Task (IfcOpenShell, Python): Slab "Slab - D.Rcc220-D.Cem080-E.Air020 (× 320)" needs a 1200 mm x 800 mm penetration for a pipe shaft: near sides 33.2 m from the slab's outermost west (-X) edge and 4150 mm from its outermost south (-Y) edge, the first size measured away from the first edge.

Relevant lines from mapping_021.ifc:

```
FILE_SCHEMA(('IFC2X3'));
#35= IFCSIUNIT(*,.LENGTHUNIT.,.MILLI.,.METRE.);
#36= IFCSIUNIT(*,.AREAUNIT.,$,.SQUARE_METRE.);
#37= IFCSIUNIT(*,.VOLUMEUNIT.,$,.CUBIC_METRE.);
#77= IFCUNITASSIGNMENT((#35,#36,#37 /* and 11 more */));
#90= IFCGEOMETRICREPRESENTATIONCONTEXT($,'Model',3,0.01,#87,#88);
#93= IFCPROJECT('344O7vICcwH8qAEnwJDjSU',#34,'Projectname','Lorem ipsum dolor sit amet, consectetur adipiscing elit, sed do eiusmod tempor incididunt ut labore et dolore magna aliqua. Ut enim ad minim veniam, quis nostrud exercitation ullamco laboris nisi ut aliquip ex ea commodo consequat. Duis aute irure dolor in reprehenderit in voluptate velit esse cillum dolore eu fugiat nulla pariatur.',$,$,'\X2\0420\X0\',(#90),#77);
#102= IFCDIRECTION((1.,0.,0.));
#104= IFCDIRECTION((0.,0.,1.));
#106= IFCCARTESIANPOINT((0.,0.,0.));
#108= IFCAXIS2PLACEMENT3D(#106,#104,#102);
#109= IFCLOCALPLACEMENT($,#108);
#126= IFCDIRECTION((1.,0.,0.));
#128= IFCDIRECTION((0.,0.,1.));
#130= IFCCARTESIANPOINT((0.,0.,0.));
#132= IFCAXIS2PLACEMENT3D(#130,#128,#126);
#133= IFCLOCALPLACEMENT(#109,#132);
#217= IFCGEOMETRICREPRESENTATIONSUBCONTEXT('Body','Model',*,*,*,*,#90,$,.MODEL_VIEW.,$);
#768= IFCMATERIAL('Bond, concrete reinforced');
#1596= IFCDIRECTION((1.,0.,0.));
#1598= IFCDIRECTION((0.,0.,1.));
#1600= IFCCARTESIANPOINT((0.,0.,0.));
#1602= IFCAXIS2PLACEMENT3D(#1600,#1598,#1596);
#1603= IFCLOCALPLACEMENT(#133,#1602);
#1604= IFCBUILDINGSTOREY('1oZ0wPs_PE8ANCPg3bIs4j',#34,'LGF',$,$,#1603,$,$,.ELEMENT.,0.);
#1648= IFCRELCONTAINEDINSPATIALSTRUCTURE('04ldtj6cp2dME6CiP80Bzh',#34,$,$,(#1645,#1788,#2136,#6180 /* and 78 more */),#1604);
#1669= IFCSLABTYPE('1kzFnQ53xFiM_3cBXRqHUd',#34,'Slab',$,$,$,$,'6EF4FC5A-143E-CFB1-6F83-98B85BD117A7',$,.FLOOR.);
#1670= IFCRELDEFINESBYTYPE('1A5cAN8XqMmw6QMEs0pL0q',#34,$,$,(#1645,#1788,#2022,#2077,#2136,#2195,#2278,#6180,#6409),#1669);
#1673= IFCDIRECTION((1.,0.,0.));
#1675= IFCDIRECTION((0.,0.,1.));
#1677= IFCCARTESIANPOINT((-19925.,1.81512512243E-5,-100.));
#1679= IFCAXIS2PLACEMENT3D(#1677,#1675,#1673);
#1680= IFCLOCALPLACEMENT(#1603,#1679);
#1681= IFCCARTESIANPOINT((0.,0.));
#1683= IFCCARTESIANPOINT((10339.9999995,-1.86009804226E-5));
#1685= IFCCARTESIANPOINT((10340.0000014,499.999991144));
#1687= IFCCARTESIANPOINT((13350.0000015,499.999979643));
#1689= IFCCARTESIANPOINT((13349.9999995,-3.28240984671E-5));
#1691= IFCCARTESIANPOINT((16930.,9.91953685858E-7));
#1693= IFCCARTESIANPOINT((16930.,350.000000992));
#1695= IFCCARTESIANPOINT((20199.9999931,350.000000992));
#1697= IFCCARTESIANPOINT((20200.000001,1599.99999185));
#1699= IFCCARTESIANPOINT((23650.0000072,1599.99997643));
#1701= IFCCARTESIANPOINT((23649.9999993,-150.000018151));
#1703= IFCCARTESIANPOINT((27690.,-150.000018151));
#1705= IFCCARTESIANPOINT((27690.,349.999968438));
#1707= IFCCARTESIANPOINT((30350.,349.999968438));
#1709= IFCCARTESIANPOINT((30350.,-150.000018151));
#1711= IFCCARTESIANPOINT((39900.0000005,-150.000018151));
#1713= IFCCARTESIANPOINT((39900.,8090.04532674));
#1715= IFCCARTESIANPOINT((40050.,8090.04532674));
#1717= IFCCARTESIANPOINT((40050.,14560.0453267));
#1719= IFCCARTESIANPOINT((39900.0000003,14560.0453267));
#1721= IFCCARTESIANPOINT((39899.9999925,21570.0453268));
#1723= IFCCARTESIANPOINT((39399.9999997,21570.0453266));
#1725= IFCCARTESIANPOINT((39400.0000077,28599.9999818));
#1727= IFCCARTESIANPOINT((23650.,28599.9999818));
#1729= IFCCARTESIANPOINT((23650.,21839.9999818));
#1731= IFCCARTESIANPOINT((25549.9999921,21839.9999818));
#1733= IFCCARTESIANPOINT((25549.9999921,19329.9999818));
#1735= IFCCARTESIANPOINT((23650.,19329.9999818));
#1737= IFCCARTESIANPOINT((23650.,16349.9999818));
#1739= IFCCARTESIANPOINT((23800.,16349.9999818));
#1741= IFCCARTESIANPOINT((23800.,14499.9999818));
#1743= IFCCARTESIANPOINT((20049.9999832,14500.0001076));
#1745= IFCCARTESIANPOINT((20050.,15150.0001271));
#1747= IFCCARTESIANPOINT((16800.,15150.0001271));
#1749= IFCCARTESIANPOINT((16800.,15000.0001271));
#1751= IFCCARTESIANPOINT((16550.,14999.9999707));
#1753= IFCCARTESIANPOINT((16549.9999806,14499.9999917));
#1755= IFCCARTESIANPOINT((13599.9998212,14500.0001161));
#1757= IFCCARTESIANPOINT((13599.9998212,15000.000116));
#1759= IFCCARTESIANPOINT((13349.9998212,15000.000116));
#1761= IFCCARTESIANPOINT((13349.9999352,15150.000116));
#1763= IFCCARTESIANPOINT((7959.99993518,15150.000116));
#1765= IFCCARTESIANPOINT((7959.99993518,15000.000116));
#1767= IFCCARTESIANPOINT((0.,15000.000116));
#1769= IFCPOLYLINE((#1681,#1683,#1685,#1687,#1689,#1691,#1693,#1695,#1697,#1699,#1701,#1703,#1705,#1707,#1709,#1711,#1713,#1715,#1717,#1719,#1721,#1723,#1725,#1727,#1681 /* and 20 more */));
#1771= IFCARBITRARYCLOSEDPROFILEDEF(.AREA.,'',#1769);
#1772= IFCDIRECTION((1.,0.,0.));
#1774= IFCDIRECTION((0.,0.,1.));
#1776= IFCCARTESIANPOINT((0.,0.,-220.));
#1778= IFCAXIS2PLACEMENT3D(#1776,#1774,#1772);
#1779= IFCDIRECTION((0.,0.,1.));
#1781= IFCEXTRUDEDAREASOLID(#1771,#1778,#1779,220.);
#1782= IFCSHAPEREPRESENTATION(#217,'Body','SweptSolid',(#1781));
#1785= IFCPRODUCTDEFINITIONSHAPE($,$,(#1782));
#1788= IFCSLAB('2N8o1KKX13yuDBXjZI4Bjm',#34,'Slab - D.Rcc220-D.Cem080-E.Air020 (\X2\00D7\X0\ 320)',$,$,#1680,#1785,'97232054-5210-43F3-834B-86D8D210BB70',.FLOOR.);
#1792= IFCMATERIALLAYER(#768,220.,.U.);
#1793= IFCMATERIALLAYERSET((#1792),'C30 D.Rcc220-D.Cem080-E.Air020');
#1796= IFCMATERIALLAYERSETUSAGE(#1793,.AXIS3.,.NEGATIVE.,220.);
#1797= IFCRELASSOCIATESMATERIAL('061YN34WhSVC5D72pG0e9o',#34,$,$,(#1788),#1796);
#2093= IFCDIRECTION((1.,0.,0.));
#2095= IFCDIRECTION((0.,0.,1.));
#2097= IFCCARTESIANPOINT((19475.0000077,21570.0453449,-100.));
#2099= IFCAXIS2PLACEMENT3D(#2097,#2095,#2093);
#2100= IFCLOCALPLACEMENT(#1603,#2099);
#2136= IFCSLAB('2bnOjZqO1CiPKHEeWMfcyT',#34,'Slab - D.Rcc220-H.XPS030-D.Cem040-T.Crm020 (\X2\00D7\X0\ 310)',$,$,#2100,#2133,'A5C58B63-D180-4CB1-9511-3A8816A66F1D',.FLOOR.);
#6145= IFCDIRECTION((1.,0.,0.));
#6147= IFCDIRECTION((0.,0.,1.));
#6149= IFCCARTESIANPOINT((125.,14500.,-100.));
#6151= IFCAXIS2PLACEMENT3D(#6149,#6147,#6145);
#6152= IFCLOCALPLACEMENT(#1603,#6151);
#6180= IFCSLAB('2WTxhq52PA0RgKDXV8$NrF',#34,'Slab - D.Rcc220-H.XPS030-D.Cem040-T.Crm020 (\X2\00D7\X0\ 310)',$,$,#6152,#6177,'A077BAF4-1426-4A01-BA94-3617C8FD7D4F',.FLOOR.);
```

```python
import numpy as np
import ifcopenshell
import ifcopenshell.api.feature
import ifcopenshell.api.geometry
import ifcopenshell.api.root
import ifcopenshell.geom
import ifcopenshell.util.placement
import ifcopenshell.util.representation
import ifcopenshell.util.shape
import ifcopenshell.util.unit

model = ifcopenshell.open("mapping_021.ifc")
unit_scale = ifcopenshell.util.unit.calculate_unit_scale(model)
settings = ifcopenshell.geom.settings()


def volume(element):
    """Net volume in cubic metres, openings subtracted."""
    shape = ifcopenshell.geom.create_shape(settings, element)
    return ifcopenshell.util.shape.get_volume(shape.geometry)


slab = model.by_guid("2N8o1KKX13yuDBXjZI4Bjm")
before = volume(slab)

# Extent in the slab's own axes, in metres. The edges named are its -X and -Y sides.
slab_shape = ifcopenshell.geom.create_shape(settings, slab)
vertices = ifcopenshell.util.shape.get_vertices(slab_shape.geometry)
x_min, y_min, bottom = vertices.min(axis=0)
top = vertices[:, 2].max()

opening = ifcopenshell.api.root.create_entity(model, ifc_class="IfcOpeningElement", name="Pipe shaft opening")
context = ifcopenshell.util.representation.get_context(model, "Model", "Body", "MODEL_VIEW")
width, depth = 1.2, 0.8
outline = [(0.0, 0.0), (width, 0.0), (width, depth), (0.0, depth), (0.0, 0.0)]
# Overshoot both faces by 50 mm so the cut is clean.
shape = ifcopenshell.api.geometry.add_slab_representation(
    model, context=context, depth=top - bottom + 0.1, polyline=outline
)
ifcopenshell.api.geometry.assign_representation(model, product=opening, representation=shape)

matrix = ifcopenshell.util.placement.get_local_placement(slab.ObjectPlacement)
matrix[:, 3] = matrix @ np.append(np.array([x_min + 33.2, y_min + 4.15, bottom - 0.05]) / unit_scale, 1.0)
ifcopenshell.api.geometry.edit_object_placement(model, product=opening, matrix=matrix, is_si=False)
ifcopenshell.api.feature.add_feature(model, feature=opening, element=slab)

after = volume(slab)

print(f"slab volume {before:.3f} -> {after:.3f} m3")

model.write("mapping_021_updated.ifc")
```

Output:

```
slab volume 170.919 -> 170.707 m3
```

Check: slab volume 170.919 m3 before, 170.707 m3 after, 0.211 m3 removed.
